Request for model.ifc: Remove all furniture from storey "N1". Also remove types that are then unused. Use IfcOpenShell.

First a look at what the model holds.

```python
import ifcopenshell
import ifcopenshell.util.element

model = ifcopenshell.open("model.ifc")
print(model.schema)
storey = next(s for s in model.by_type("IfcBuildingStorey") if s.Name == "N1")
furniture = [e for e in ifcopenshell.util.element.get_decomposition(storey) if e.is_a("IfcFurnishingElement")]
seen = {}
for e in furniture:
    element_type = ifcopenshell.util.element.get_type(e)
    name = element_type.Name if element_type not in (None, e) else None
    seen[name] = seen.get(name, 0) + 1
for name, count in sorted(seen.items(), key=str):
    print(count, "x", name)
```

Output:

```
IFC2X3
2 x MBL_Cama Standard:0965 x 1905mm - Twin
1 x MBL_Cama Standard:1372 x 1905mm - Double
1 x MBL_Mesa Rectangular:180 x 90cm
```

```python
import ifcopenshell
import ifcopenshell.api.root
import ifcopenshell.util.element

model = ifcopenshell.open("model.ifc")

storey = next(s for s in model.by_type("IfcBuildingStorey") if s.Name == "N1")
furniture = [e for e in ifcopenshell.util.element.get_decomposition(storey) if e.is_a("IfcFurnishingElement")]
types = {ifcopenshell.util.element.get_type(e) for e in furniture} - {None, *furniture}

for e in furniture:
    ifcopenshell.api.root.remove_product(model, product=e)
print(len(furniture), "removed")

unused = [t for t in types if not ifcopenshell.util.element.get_types(t)]
for t in unused:
    ifcopenshell.api.root.remove_product(model, product=t)
print(len(unused), "unused types removed")

model.write("model_v2.ifc")
```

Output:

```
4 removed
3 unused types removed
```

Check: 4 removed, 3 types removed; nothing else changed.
